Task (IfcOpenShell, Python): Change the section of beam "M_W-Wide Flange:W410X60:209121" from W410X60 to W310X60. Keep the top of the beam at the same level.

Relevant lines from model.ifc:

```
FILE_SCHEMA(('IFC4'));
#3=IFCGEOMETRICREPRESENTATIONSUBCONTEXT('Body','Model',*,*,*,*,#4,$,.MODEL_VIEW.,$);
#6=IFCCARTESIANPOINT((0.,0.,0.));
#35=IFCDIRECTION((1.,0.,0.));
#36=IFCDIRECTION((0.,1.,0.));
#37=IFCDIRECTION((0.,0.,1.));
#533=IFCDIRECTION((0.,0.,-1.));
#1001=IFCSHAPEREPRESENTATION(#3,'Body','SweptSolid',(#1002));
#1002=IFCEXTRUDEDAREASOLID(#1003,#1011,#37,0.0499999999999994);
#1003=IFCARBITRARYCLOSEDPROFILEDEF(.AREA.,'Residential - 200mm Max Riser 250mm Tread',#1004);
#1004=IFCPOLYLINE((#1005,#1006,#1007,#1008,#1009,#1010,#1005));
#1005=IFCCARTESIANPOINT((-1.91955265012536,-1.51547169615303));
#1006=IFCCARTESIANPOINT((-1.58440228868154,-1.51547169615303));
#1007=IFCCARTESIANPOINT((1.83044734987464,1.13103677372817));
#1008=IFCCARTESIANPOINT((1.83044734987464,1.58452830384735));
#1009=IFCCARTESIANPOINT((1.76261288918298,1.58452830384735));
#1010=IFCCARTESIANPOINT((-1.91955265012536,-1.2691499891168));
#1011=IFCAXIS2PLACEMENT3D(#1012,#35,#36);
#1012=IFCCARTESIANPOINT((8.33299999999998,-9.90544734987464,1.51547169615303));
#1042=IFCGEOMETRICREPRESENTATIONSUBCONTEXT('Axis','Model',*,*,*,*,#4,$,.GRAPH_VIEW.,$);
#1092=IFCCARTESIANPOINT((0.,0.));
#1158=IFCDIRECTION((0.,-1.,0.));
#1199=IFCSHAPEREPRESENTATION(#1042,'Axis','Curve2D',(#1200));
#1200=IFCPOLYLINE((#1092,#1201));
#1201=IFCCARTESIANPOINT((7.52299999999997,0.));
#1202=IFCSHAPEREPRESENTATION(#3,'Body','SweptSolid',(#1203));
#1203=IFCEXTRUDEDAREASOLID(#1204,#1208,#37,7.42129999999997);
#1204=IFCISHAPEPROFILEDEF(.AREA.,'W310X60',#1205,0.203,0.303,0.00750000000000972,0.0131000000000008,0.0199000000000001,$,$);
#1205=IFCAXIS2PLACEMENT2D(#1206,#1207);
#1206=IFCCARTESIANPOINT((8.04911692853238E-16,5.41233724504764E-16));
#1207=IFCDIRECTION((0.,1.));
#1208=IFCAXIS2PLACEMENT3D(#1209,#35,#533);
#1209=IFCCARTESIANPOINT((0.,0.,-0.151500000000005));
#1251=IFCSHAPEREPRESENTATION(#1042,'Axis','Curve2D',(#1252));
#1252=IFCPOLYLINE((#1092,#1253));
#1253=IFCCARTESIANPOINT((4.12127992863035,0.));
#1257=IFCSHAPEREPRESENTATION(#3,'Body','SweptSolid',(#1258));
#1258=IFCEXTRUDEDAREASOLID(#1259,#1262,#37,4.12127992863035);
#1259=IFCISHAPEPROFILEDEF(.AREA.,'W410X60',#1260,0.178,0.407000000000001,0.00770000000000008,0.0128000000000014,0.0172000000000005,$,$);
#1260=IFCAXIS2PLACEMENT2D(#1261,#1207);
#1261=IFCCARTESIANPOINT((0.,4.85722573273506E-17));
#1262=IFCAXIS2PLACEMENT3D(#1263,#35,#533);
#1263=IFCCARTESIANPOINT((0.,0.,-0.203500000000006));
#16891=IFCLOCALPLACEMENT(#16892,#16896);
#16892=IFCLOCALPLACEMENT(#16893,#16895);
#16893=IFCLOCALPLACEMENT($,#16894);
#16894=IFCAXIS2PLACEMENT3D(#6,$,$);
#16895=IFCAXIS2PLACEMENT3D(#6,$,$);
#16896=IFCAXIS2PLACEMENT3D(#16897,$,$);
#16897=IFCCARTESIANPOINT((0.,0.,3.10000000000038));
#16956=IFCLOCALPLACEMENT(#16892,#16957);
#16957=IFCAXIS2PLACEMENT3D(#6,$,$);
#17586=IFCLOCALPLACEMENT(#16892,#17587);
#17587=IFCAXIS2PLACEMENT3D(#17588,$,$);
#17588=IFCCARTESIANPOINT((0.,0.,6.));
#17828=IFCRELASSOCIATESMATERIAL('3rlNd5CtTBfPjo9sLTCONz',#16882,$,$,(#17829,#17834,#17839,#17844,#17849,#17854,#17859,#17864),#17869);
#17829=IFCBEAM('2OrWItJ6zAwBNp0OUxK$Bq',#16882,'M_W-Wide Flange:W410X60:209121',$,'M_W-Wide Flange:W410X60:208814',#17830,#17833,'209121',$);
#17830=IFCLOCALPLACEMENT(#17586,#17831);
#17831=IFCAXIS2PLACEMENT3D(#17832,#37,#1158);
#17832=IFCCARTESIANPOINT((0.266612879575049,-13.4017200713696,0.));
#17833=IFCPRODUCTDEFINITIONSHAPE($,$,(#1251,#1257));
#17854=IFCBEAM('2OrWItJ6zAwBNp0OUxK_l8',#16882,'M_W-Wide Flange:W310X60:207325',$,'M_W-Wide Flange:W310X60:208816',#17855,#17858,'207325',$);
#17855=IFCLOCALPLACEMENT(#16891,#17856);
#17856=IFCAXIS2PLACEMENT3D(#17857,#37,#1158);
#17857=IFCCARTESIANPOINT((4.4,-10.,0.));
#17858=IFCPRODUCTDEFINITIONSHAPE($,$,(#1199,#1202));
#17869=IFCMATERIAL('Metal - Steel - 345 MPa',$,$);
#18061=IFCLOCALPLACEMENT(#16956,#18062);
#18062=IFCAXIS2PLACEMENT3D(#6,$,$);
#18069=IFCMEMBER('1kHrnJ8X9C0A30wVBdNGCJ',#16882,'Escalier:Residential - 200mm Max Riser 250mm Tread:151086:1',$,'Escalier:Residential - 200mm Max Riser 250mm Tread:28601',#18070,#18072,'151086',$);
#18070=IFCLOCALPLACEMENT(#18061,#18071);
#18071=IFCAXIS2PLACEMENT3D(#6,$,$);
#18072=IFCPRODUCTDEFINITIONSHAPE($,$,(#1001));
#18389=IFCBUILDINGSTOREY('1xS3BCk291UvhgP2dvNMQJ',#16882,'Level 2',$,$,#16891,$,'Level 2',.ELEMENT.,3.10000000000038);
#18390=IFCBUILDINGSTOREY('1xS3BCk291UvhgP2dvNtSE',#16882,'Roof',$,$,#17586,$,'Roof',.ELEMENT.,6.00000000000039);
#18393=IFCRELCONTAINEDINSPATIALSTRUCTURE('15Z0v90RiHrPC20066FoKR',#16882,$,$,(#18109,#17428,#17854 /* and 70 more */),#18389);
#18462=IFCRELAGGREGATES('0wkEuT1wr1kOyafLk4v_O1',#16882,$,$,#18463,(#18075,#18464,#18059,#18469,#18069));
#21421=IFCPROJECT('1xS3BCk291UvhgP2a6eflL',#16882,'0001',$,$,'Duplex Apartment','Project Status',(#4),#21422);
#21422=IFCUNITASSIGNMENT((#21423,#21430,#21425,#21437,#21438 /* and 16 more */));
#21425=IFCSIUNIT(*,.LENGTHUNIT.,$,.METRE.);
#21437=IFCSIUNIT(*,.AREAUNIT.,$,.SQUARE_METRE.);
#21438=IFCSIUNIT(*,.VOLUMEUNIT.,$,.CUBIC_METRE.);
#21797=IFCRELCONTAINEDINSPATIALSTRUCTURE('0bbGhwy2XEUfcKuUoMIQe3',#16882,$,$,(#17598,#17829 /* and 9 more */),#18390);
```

```python
import ifcopenshell
import ifcopenshell.util.element
import ifcopenshell.util.representation

model = ifcopenshell.open("model.ifc")

member = model.by_guid("2OrWItJ6zAwBNp0OUxK$Bq")
source = next(p for p in model.by_type("IfcIShapeProfileDef") if p.ProfileName == "W310X60")

body = ifcopenshell.util.representation.get_representation(member, "Model", "Body")
solid = body.Items[0]
old_profile = solid.SweptArea

# Copy the section's sizes but keep this member's own profile position.
profile = ifcopenshell.util.element.copy(model, source)
# Profiles are centred, so shift by half the change in depth to hold the top.
shift = (old_profile.OverallDepth - profile.OverallDepth) / 2
x, y = old_profile.Position.Location.Coordinates
up = (-1.0, 0.0)  # upwards, in the solid's own plane
location = model.createIfcCartesianPoint((x + up[0] * shift, y + up[1] * shift))
profile.Position = model.createIfcAxis2Placement2D(location, old_profile.Position.RefDirection)
solid.SweptArea = profile
if not model.get_total_inverses(old_profile):
    ifcopenshell.util.element.remove_deep2(model, old_profile)
member.Name = member.Name.replace("W410X60", "W310X60")
member.ObjectType = member.ObjectType.replace("W410X60", "W310X60")

print(solid.SweptArea)

model.write("model_updated.ifc")
```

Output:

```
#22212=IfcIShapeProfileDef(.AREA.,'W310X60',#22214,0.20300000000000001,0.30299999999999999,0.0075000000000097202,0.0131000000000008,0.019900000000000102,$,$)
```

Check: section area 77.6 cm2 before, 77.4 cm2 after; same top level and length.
